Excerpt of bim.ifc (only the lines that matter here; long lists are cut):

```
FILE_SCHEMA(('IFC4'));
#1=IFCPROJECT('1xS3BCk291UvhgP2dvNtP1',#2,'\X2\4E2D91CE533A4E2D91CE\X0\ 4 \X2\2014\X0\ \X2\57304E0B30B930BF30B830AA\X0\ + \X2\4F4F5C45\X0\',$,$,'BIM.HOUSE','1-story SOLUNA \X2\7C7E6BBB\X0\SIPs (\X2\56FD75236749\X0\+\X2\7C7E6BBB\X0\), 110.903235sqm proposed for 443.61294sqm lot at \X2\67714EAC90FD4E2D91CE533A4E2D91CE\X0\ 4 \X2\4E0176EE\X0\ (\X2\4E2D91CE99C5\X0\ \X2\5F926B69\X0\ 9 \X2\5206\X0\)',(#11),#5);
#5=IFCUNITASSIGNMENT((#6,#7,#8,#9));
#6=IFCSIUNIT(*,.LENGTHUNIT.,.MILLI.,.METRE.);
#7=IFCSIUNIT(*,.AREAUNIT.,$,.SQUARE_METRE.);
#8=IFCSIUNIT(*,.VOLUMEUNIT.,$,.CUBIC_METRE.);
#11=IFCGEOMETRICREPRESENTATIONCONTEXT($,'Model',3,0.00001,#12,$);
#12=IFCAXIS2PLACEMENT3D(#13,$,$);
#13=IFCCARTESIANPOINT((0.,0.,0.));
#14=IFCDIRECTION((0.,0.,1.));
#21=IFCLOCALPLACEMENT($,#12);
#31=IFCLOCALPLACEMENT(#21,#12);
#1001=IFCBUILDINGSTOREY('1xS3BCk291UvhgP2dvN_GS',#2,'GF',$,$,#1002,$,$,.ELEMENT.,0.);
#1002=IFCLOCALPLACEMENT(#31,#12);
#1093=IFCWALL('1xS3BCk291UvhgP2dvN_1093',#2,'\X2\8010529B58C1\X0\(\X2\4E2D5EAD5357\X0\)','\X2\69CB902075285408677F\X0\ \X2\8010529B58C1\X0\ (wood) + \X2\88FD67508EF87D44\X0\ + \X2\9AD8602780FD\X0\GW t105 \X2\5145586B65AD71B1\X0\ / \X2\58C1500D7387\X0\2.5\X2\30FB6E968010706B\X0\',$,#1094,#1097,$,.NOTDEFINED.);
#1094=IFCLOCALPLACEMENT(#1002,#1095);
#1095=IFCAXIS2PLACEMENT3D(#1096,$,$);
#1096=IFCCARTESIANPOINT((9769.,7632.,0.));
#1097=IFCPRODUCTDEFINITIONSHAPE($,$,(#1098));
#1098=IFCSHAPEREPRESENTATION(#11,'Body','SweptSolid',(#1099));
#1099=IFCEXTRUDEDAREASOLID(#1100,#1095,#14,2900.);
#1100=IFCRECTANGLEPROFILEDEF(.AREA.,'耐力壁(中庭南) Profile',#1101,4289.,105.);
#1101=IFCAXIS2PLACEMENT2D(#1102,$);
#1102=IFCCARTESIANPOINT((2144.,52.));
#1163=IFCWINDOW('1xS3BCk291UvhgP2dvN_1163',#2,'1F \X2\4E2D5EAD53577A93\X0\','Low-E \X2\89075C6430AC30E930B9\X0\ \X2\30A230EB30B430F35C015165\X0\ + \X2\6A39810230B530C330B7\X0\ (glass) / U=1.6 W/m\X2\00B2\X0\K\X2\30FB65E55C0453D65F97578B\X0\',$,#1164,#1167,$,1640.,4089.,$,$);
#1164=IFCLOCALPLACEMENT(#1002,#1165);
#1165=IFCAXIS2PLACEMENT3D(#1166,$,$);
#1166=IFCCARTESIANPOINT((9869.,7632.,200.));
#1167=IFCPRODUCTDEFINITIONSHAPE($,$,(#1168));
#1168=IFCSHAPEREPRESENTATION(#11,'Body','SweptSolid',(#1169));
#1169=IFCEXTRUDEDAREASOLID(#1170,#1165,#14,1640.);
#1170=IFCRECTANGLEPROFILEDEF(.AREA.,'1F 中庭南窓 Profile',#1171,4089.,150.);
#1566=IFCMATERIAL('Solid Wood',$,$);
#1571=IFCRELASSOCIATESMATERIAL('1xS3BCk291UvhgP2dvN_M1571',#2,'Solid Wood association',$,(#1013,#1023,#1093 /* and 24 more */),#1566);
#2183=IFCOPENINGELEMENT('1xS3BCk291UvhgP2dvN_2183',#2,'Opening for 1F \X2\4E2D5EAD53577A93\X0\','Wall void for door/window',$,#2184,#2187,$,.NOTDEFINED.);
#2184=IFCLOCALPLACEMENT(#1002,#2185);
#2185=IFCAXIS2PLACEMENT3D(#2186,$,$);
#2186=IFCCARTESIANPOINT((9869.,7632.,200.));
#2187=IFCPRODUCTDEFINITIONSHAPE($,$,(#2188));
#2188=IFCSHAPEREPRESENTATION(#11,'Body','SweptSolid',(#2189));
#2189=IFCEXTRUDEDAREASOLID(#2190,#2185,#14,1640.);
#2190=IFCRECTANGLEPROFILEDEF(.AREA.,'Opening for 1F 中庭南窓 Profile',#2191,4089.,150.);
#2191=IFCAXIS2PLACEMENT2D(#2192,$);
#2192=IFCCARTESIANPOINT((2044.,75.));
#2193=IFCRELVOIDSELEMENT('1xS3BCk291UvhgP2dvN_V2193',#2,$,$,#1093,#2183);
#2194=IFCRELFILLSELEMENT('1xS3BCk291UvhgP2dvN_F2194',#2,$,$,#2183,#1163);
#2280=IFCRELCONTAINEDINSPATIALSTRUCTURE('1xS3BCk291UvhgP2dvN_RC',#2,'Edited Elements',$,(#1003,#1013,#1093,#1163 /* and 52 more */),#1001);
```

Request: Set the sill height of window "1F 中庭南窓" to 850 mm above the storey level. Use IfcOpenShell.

```python
import numpy as np
import ifcopenshell
import ifcopenshell.api.geometry
import ifcopenshell.geom
import ifcopenshell.util.element
import ifcopenshell.util.placement
import ifcopenshell.util.shape
import ifcopenshell.util.unit

model = ifcopenshell.open("bim.ifc")
unit_scale = ifcopenshell.util.unit.calculate_unit_scale(model)

window = model.by_id(1163)
opening = window.FillsVoids[0].RelatingOpeningElement
storey = ifcopenshell.util.element.get_container(window, ifc_class="IfcBuildingStorey")
level = ifcopenshell.util.placement.get_local_placement(storey.ObjectPlacement)[2, 3]

# The opening's origin need not be at the sill, so measure its lowest point.
shape = ifcopenshell.geom.create_shape(ifcopenshell.geom.settings(), opening)
bottom = ifcopenshell.util.shape.get_shape_bottom_elevation(shape, shape.geometry) / unit_scale
dz = level + 0.85 / unit_scale - bottom

shift = np.array([0.0, 0.0, dz])
# The window is not placed relative to its opening, so move both.
for product in (opening, window):
    matrix = ifcopenshell.util.placement.get_local_placement(product.ObjectPlacement)
    matrix[:3, 3] += shift
    ifcopenshell.api.geometry.edit_object_placement(model, product=product, matrix=matrix, is_si=False)

print(f"moved by {dz * unit_scale:+.3f} m")

model.write("bim_updated.ifc")
```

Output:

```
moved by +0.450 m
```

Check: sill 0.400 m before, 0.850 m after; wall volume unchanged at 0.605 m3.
